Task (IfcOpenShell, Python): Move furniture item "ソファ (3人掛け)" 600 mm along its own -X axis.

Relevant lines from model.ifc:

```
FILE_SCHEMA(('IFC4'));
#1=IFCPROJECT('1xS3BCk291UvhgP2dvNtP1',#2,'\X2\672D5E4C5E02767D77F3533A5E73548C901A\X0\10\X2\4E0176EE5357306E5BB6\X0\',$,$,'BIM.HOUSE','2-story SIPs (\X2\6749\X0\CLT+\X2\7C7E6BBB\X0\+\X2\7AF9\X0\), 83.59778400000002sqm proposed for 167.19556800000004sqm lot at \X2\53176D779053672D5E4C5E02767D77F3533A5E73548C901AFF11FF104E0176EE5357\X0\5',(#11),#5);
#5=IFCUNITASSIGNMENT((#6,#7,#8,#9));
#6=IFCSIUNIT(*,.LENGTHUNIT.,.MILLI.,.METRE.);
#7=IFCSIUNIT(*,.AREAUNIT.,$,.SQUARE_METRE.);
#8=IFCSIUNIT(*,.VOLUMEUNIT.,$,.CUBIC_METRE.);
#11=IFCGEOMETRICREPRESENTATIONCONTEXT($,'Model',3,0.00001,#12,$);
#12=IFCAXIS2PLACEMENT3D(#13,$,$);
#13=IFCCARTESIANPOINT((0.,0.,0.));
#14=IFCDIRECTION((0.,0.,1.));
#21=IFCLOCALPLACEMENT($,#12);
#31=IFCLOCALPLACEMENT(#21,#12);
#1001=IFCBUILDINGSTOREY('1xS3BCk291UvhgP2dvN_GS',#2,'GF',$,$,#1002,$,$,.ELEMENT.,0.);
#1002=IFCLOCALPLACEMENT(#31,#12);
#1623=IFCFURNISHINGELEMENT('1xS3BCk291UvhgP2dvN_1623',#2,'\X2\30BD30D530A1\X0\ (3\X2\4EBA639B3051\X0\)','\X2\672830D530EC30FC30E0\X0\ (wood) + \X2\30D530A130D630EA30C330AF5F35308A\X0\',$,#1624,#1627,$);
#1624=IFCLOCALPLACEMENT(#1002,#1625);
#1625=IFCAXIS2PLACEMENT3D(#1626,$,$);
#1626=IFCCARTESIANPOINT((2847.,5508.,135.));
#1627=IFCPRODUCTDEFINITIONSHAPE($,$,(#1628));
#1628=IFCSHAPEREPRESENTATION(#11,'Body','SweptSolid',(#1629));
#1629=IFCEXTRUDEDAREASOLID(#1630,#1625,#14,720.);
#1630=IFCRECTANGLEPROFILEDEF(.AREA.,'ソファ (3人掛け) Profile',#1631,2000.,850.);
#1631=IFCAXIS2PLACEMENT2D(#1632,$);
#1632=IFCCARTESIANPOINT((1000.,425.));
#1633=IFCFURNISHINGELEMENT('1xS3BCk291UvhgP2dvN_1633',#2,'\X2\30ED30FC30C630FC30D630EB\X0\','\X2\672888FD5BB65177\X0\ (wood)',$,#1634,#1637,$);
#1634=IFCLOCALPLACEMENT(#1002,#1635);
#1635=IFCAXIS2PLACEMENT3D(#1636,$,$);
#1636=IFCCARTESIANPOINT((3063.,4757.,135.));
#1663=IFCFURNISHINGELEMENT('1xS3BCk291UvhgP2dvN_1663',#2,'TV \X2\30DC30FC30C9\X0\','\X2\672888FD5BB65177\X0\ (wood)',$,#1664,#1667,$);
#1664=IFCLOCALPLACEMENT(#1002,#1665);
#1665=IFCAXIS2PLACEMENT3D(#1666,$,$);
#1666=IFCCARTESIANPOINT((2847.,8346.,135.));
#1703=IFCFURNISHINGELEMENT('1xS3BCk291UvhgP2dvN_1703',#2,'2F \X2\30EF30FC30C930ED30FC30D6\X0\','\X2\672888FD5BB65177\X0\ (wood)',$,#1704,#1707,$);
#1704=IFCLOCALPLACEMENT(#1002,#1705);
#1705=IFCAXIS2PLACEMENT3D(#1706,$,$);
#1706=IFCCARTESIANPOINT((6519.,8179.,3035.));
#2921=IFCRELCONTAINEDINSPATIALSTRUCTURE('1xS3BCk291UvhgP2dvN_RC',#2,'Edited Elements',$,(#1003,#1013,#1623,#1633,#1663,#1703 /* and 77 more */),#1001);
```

```python
import ifcopenshell
import ifcopenshell.api.geometry
import ifcopenshell.util.placement
import ifcopenshell.util.unit

model = ifcopenshell.open("model.ifc")
unit_scale = ifcopenshell.util.unit.calculate_unit_scale(model)

item = model.by_guid("1xS3BCk291UvhgP2dvN_1623")
matrix = ifcopenshell.util.placement.get_local_placement(item.ObjectPlacement)
matrix[:3, 3] -= matrix[:3, 0] * 0.6 / unit_scale
ifcopenshell.api.geometry.edit_object_placement(model, product=item, matrix=matrix, is_si=False)

print(ifcopenshell.util.placement.get_local_placement(item.ObjectPlacement).round(3) + 0.0)

model.write("model_v2.ifc")
```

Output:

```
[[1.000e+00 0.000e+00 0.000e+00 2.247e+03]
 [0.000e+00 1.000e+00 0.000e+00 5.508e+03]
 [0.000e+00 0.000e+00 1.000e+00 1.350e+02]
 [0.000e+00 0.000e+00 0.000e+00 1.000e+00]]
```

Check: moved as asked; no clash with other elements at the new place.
